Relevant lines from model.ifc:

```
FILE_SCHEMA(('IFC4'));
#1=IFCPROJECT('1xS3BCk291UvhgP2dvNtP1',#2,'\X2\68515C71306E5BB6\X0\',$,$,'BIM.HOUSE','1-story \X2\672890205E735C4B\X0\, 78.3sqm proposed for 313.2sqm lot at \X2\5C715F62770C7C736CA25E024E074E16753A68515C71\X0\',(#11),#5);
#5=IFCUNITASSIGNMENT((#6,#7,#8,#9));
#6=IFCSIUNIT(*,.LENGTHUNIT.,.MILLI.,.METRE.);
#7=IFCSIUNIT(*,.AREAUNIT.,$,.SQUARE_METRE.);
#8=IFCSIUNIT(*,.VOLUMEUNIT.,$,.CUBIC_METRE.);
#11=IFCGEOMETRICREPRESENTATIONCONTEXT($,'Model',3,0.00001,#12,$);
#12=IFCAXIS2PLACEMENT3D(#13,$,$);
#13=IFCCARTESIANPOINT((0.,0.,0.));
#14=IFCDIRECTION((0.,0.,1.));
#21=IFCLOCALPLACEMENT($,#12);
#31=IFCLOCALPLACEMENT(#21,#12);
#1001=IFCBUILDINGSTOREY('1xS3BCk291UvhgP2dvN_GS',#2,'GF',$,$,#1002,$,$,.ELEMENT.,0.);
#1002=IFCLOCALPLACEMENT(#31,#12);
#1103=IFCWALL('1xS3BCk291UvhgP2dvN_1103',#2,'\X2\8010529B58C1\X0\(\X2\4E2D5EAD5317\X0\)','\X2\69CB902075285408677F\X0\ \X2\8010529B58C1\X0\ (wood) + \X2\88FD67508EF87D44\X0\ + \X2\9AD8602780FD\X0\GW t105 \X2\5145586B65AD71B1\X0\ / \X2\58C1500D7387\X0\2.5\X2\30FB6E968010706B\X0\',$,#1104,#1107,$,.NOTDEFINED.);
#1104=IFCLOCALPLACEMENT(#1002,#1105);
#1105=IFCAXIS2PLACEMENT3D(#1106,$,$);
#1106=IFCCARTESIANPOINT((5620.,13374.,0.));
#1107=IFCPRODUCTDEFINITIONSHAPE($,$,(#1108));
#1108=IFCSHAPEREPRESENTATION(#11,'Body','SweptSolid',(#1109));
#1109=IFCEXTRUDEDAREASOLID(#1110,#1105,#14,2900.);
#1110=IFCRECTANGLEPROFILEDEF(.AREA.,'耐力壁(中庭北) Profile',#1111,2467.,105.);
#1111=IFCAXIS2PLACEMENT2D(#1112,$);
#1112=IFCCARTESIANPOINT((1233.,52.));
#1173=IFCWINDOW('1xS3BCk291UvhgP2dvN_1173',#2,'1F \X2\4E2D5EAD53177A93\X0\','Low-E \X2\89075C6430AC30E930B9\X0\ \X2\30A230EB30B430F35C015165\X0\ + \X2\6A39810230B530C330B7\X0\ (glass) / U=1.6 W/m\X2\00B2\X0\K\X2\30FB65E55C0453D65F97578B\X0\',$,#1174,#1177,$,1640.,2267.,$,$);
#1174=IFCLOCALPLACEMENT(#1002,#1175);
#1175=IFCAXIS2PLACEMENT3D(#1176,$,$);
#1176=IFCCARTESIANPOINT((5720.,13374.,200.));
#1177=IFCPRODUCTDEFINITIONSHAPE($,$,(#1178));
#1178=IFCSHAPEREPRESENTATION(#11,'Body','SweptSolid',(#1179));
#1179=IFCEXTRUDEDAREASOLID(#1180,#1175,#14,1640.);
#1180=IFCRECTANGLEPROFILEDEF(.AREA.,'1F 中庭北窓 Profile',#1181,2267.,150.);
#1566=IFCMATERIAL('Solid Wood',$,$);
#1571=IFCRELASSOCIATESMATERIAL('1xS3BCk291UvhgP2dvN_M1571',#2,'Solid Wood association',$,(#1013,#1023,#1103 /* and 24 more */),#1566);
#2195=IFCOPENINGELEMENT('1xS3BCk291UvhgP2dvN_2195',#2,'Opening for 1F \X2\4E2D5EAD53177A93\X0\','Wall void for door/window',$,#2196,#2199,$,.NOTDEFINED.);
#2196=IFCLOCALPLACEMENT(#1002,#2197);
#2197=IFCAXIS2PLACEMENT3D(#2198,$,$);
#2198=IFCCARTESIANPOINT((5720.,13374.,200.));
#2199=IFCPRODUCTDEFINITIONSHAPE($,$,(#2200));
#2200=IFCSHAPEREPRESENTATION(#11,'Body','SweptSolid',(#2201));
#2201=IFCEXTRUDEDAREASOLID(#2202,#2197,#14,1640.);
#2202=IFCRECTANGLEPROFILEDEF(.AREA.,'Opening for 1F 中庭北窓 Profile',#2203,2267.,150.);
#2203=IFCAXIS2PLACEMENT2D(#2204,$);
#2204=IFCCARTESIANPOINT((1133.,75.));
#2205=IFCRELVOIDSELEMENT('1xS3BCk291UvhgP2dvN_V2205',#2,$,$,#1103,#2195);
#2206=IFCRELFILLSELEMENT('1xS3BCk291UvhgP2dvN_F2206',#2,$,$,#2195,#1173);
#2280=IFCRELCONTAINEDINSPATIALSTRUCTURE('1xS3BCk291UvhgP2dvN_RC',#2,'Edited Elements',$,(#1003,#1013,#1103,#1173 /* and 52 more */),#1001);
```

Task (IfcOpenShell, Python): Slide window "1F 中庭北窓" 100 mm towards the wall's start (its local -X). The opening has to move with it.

```python
import ifcopenshell
import ifcopenshell.api.geometry
import ifcopenshell.util.placement

model = ifcopenshell.open("model.ifc")

window = model.by_id(1173)
opening = window.FillsVoids[0].RelatingOpeningElement
wall = opening.VoidsElements[0].RelatingBuildingElement

wall_matrix = ifcopenshell.util.placement.get_local_placement(wall.ObjectPlacement)
shift = wall_matrix[:3, 0] * -100.0
before = ifcopenshell.util.placement.get_local_placement(window.ObjectPlacement)[:3, 3].copy()

# The window is not placed relative to its opening, so move both.
for product in (opening, window):
    matrix = ifcopenshell.util.placement.get_local_placement(product.ObjectPlacement)
    matrix[:3, 3] += shift
    ifcopenshell.api.geometry.edit_object_placement(model, product=product, matrix=matrix, is_si=False)

after = ifcopenshell.util.placement.get_local_placement(window.ObjectPlacement)[:3, 3]
print("window moved by", (after - before).round(3) + 0.0)

model.write("model-out.ifc")
```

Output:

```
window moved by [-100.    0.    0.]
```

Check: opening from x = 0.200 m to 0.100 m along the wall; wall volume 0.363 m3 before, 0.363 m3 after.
